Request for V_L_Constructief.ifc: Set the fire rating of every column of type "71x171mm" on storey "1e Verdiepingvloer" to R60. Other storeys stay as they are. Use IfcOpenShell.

First a look at what the model holds.

```python
import ifcopenshell
import ifcopenshell.util.element

model = ifcopenshell.open("V_L_Constructief.ifc")
print(model.schema)
storey = next(s for s in model.by_type("IfcBuildingStorey") if s.Name == "1e Verdiepingvloer")
columns = [e for e in ifcopenshell.util.element.get_decomposition(storey) if e.is_a("IfcColumn")]
seen = {}
for e in columns:
    element_type = ifcopenshell.util.element.get_type(e)
    key = (element_type.Name if element_type != e and element_type else None, ifcopenshell.util.element.get_pset(e, "Pset_ColumnCommon", "FireRating"))
    seen[key] = seen.get(key, 0) + 1
for (name, value), count in sorted(seen.items(), key=str):
    print(count, "x", name, "|", value)
```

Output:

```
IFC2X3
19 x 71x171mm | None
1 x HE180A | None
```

```python
import ifcopenshell
import ifcopenshell.api.pset
import ifcopenshell.util.element

model = ifcopenshell.open("V_L_Constructief.ifc")

storey = next(s for s in model.by_type("IfcBuildingStorey") if s.Name == "1e Verdiepingvloer")
columns = [e for e in ifcopenshell.util.element.get_decomposition(storey) if e.is_a("IfcColumn")]

count = 0
for e in columns:
    element_type = ifcopenshell.util.element.get_type(e)
    if element_type in (None, e) or element_type.Name != "71x171mm":
        continue
    found = ifcopenshell.util.element.get_pset(e, "Pset_ColumnCommon", should_inherit=False)
    if found:
        pset = model.by_id(found["id"])
        if len(ifcopenshell.util.element.get_elements_by_pset(pset)) > 1:
            pset = ifcopenshell.api.pset.unshare_pset(model, products=[e], pset=pset)[0]
    else:
        pset = ifcopenshell.api.pset.add_pset(model, product=e, name="Pset_ColumnCommon")
    ifcopenshell.api.pset.edit_pset(model, pset=pset, properties={"FireRating": "R60"})
    count += 1

print(count, "columns updated")

model.write("V_L_Constructief_updated.ifc")
```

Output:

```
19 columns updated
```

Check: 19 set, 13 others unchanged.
